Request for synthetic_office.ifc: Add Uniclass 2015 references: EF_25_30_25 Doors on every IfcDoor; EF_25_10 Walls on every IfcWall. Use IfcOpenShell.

First a look at what the model holds.

```python
import ifcopenshell

model = ifcopenshell.open("synthetic_office.ifc")
print(model.schema)
print("classifications:", [c.Name for c in model.by_type("IfcClassification")])
for ifc_class in ("IfcDoor", "IfcRoof", "IfcStair", "IfcWall", "IfcWindow"):
    print(ifc_class, len(model.by_type(ifc_class)))
```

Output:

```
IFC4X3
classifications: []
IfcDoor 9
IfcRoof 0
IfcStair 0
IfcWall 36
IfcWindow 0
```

```python
import ifcopenshell
import ifcopenshell.api.classification

model = ifcopenshell.open("synthetic_office.ifc")

system = ifcopenshell.api.classification.add_classification(model, classification="Uniclass 2015")

codes = {
    "IfcDoor": ("EF_25_30_25", "Doors"),
    "IfcWall": ("EF_25_10", "Walls"),
}
for ifc_class, (code, name) in codes.items():
    products = model.by_type(ifc_class)
    ifcopenshell.api.classification.add_reference(
        model, products=products, classification=system, identification=code, name=name
    )
    print(code, len(products))

model.write("synthetic_office_updated.ifc")
```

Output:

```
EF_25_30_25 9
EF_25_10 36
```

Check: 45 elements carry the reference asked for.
